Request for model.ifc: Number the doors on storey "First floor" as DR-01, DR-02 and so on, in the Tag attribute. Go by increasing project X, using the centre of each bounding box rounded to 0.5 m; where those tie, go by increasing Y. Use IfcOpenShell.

First a look at what the model holds.

```python
import ifcopenshell
import ifcopenshell.util.element
import ifcopenshell.util.placement

model = ifcopenshell.open("model.ifc")
print(model.schema)
storey = next(s for s in model.by_type("IfcBuildingStorey") if s.Name == "First floor")
doors = [e for e in ifcopenshell.util.element.get_decomposition(storey) if e.is_a("IfcDoor")]
for e in sorted(doors, key=lambda e: e.id()):
    origin = ifcopenshell.util.placement.get_local_placement(e.ObjectPlacement)[:3, 3]
    print(e.id(), e.Tag, e.Name, origin.round(2) + 0.0, sep=" | ")
```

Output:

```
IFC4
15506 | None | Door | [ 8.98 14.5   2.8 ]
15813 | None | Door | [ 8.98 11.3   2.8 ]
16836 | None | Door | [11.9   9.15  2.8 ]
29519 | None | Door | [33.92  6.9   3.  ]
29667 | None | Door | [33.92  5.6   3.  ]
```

```python
import ifcopenshell
import ifcopenshell.geom
import ifcopenshell.util.element
import ifcopenshell.util.shape

model = ifcopenshell.open("model.ifc")
settings = ifcopenshell.geom.settings()
settings.set("use-world-coords", True)


def centre(element):
    shape = ifcopenshell.geom.create_shape(settings, element)
    return ifcopenshell.util.shape.get_bbox_centroid(shape.geometry)


storey = next(s for s in model.by_type("IfcBuildingStorey") if s.Name == "First floor")
doors = [e for e in ifcopenshell.util.element.get_decomposition(storey) if e.is_a("IfcDoor")]

# Insertion points can sit at a corner or the storey origin, so sort by the geometry (in metres).
centres = {e: centre(e) for e in doors}
doors.sort(key=lambda e: (round(centres[e][0] / 0.5), centres[e][1]))

for i, e in enumerate(doors, start=1):
    number = f"DR-{i:02d}"
    e.Tag = number
    print(e.id(), number)

model.write("model-out.ifc")
```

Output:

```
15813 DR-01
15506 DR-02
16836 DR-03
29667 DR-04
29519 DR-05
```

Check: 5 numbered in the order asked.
